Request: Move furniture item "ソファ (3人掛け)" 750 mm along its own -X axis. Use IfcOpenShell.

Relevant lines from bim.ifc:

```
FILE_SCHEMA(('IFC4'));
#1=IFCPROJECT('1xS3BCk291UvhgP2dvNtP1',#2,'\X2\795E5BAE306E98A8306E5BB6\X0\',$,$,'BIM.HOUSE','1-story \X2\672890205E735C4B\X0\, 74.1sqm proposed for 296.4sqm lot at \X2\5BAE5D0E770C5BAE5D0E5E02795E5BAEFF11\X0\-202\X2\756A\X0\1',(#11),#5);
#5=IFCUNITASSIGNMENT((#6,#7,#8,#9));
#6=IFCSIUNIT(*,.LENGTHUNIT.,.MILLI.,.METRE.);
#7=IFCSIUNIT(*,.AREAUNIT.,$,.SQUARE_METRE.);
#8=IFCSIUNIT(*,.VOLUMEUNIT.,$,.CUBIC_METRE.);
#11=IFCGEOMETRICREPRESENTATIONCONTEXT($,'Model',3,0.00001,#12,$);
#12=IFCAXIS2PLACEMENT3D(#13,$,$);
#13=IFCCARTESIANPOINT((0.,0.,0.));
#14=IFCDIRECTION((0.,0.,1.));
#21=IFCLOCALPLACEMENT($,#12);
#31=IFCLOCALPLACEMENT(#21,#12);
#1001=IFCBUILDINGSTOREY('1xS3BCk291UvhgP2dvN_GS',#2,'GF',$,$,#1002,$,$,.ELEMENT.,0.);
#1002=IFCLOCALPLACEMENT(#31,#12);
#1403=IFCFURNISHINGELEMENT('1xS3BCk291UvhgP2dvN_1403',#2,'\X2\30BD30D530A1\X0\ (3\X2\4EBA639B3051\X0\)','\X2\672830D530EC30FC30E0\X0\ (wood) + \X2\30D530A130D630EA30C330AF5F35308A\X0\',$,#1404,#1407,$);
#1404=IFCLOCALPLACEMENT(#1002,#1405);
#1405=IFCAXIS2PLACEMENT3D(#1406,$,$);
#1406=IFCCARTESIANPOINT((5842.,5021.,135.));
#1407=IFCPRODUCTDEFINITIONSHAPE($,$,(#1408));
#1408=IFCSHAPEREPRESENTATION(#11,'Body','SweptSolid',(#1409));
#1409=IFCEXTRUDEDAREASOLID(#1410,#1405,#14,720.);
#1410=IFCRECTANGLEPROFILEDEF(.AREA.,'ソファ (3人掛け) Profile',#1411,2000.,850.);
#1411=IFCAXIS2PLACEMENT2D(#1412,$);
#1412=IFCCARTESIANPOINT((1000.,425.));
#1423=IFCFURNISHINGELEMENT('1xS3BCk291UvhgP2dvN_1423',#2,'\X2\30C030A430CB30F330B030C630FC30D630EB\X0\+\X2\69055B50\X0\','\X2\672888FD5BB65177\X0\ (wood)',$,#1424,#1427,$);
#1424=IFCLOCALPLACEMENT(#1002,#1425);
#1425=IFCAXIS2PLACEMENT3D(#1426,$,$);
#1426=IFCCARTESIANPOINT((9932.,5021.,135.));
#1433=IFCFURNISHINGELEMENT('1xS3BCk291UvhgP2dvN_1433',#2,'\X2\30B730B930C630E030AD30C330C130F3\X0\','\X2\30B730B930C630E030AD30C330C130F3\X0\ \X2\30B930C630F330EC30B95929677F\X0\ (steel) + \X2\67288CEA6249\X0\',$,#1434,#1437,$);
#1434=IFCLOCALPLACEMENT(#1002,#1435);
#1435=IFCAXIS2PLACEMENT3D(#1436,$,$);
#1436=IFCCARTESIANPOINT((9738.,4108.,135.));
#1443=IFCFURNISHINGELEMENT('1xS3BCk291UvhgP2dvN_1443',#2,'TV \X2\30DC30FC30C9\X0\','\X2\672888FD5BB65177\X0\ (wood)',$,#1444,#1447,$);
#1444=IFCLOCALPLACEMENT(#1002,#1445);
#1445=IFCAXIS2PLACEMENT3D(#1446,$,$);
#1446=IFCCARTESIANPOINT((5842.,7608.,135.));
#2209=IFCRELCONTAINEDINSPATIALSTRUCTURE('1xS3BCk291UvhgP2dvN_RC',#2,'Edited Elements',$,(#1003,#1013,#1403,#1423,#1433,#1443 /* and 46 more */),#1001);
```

```python
import ifcopenshell
import ifcopenshell.api.geometry
import ifcopenshell.util.placement
import ifcopenshell.util.unit

model = ifcopenshell.open("bim.ifc")
unit_scale = ifcopenshell.util.unit.calculate_unit_scale(model)

item = model.by_guid("1xS3BCk291UvhgP2dvN_1403")
matrix = ifcopenshell.util.placement.get_local_placement(item.ObjectPlacement)
matrix[:3, 3] -= matrix[:3, 0] * 0.75 / unit_scale
ifcopenshell.api.geometry.edit_object_placement(model, product=item, matrix=matrix, is_si=False)

print(ifcopenshell.util.placement.get_local_placement(item.ObjectPlacement).round(3) + 0.0)

model.write("bim_updated.ifc")
```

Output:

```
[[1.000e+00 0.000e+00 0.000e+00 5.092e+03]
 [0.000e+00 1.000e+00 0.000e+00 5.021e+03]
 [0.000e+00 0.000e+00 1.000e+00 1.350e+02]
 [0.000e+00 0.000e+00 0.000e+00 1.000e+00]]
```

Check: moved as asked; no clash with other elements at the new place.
